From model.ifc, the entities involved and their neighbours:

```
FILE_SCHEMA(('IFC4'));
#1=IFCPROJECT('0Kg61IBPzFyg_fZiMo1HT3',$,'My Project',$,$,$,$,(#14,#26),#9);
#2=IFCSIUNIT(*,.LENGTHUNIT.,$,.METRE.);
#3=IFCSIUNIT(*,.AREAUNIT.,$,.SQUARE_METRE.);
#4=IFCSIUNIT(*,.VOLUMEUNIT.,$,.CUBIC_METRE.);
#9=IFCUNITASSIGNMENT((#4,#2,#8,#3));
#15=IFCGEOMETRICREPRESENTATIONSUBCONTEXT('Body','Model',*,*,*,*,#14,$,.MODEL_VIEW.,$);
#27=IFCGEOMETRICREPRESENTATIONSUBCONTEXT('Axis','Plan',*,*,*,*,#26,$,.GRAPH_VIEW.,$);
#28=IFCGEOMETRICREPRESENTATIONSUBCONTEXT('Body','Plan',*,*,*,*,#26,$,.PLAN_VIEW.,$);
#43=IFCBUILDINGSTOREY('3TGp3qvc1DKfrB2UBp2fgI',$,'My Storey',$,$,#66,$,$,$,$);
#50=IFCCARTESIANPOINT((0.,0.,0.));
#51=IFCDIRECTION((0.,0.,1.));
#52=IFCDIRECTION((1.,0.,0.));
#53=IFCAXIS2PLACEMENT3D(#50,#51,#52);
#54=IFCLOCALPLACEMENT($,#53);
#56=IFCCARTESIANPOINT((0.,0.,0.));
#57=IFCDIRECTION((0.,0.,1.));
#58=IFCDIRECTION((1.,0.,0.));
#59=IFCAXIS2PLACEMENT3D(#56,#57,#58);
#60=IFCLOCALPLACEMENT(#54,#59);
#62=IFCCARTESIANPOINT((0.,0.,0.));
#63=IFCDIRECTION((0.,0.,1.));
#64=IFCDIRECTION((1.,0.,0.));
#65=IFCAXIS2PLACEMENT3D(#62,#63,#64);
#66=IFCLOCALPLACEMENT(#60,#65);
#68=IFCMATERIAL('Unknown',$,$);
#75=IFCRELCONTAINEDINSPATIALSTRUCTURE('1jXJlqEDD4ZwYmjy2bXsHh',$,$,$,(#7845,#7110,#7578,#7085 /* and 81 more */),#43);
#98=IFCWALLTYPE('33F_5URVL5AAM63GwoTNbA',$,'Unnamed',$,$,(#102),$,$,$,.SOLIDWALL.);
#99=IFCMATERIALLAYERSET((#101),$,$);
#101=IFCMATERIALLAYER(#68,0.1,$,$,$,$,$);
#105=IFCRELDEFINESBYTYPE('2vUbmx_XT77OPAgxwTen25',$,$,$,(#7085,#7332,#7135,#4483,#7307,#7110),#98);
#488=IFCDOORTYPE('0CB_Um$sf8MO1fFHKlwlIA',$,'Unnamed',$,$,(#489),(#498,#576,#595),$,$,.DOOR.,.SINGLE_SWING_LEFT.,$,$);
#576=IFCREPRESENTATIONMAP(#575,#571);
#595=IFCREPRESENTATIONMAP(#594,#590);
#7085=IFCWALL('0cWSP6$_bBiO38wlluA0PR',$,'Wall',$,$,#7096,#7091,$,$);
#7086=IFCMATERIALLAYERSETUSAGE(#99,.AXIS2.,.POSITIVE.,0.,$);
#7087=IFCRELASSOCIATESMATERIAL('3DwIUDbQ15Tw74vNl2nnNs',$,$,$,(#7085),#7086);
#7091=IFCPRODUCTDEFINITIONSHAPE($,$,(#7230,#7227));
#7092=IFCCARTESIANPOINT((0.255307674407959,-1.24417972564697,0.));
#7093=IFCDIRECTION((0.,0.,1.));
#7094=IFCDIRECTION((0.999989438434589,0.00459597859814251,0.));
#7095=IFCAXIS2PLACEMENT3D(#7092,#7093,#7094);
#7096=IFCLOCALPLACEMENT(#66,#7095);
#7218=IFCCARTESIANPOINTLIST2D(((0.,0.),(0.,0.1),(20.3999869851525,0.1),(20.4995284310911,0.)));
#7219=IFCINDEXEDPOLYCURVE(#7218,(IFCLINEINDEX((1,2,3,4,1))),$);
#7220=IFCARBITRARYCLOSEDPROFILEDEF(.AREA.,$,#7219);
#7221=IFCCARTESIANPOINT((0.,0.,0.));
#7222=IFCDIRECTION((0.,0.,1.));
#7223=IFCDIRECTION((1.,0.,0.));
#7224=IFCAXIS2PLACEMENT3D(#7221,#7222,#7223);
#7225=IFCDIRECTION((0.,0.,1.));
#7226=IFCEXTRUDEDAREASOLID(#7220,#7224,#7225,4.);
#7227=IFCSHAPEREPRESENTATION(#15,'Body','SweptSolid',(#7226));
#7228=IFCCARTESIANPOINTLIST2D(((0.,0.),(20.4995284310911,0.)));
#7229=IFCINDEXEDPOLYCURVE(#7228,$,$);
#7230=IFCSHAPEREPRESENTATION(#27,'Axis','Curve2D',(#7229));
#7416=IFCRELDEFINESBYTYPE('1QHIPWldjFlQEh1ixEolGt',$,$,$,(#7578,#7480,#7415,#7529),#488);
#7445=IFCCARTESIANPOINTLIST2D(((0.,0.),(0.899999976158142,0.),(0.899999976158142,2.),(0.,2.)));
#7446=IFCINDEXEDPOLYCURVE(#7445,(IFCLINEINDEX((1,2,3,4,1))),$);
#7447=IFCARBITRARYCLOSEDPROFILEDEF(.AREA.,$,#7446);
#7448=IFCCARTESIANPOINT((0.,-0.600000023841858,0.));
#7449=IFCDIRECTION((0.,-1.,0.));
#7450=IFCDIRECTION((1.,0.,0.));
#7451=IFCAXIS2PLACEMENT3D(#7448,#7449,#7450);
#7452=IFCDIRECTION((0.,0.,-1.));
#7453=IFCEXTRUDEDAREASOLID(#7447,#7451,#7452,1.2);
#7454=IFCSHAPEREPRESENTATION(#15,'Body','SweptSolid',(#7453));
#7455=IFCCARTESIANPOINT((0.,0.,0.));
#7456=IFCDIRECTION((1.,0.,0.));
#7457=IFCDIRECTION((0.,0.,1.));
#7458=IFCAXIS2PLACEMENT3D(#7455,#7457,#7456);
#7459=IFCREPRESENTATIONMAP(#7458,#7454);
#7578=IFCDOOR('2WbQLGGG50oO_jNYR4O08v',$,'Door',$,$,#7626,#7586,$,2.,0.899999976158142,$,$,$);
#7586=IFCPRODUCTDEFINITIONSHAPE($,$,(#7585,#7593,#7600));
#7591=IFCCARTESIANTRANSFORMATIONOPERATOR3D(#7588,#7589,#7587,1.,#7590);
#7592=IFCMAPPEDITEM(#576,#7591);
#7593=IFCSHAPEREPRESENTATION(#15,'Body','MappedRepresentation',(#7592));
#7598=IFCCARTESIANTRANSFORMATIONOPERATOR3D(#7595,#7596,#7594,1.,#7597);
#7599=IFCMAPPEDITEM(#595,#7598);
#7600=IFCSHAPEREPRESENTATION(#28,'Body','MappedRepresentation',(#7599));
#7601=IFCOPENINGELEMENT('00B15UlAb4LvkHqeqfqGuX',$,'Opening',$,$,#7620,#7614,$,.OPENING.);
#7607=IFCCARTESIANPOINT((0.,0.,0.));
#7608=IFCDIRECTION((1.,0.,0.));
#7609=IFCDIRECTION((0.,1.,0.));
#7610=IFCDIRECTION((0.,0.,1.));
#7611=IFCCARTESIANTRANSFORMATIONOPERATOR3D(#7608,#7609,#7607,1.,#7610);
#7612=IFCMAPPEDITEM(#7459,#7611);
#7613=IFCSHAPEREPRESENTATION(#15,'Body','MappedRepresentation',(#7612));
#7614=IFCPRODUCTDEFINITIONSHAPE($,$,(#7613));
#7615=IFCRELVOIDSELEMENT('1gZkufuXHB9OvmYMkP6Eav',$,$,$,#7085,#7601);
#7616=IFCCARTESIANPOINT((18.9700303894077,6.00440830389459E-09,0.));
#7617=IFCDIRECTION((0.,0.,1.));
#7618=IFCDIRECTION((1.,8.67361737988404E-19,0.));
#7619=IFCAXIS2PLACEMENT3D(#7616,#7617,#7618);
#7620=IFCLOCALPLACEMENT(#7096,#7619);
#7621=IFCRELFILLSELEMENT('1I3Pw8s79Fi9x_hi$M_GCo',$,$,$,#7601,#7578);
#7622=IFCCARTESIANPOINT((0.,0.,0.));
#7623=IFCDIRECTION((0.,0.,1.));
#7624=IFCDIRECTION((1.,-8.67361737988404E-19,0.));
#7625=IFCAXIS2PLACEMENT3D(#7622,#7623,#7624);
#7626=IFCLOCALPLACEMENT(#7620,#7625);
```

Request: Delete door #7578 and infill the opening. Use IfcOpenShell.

```python
import ifcopenshell
import ifcopenshell.api.feature
import ifcopenshell.api.root
import ifcopenshell.geom
import ifcopenshell.util.shape

model = ifcopenshell.open("model.ifc")
settings = ifcopenshell.geom.settings()


def volume(element):
    """Net volume in cubic metres, openings subtracted."""
    shape = ifcopenshell.geom.create_shape(settings, element)
    return ifcopenshell.util.shape.get_volume(shape.geometry)


door = model.by_guid("2WbQLGGG50oO_jNYR4O08v")
opening = door.FillsVoids[0].RelatingOpeningElement
wall = opening.VoidsElements[0].RelatingBuildingElement
before = volume(wall)

ifcopenshell.api.root.remove_product(model, product=door)
ifcopenshell.api.feature.remove_feature(model, feature=opening)

after = volume(wall)

print(f"wall volume {before:.3f} -> {after:.3f} m3")

model.write("model_v2.ifc")
```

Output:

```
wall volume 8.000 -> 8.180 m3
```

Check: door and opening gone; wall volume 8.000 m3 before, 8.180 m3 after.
